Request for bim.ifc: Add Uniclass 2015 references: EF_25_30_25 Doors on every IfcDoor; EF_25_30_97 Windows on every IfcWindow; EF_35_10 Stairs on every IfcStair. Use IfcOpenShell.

First a look at what the model holds.

```python
import ifcopenshell

model = ifcopenshell.open("bim.ifc")
print(model.schema)
print("classifications:", [c.Name for c in model.by_type("IfcClassification")])
for ifc_class in ("IfcDoor", "IfcRoof", "IfcStair", "IfcWall", "IfcWindow"):
    print(ifc_class, len(model.by_type(ifc_class)))
```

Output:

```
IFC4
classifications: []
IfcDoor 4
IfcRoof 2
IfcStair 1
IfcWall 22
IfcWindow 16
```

```python
import ifcopenshell
import ifcopenshell.api.classification

model = ifcopenshell.open("bim.ifc")

system = ifcopenshell.api.classification.add_classification(model, classification="Uniclass 2015")

codes = {
    "IfcDoor": ("EF_25_30_25", "Doors"),
    "IfcWindow": ("EF_25_30_97", "Windows"),
    "IfcStair": ("EF_35_10", "Stairs"),
}
for ifc_class, (code, name) in codes.items():
    products = model.by_type(ifc_class)
    ifcopenshell.api.classification.add_reference(
        model, products=products, classification=system, identification=code, name=name
    )
    print(code, len(products))

model.write("bim_rev.ifc")
```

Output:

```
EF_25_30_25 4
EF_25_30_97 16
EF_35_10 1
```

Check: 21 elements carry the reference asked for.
